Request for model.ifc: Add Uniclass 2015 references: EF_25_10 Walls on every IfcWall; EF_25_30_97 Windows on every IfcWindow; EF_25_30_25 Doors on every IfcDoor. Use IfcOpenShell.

First a look at what the model holds.

```python
import ifcopenshell

model = ifcopenshell.open("model.ifc")
print(model.schema)
print("classifications:", [c.Name for c in model.by_type("IfcClassification")])
for ifc_class in ("IfcDoor", "IfcRoof", "IfcStair", "IfcWall", "IfcWindow"):
    print(ifc_class, len(model.by_type(ifc_class)))
```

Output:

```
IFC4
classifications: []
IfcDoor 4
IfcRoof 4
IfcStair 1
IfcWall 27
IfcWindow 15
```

```python
import ifcopenshell
import ifcopenshell.api.classification

model = ifcopenshell.open("model.ifc")

system = ifcopenshell.api.classification.add_classification(model, classification="Uniclass 2015")

codes = {
    "IfcWall": ("EF_25_10", "Walls"),
    "IfcWindow": ("EF_25_30_97", "Windows"),
    "IfcDoor": ("EF_25_30_25", "Doors"),
}
for ifc_class, (code, name) in codes.items():
    products = model.by_type(ifc_class)
    ifcopenshell.api.classification.add_reference(
        model, products=products, classification=system, identification=code, name=name
    )
    print(code, len(products))

model.write("model_edited.ifc")
```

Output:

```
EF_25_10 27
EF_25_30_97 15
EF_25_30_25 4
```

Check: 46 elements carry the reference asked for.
